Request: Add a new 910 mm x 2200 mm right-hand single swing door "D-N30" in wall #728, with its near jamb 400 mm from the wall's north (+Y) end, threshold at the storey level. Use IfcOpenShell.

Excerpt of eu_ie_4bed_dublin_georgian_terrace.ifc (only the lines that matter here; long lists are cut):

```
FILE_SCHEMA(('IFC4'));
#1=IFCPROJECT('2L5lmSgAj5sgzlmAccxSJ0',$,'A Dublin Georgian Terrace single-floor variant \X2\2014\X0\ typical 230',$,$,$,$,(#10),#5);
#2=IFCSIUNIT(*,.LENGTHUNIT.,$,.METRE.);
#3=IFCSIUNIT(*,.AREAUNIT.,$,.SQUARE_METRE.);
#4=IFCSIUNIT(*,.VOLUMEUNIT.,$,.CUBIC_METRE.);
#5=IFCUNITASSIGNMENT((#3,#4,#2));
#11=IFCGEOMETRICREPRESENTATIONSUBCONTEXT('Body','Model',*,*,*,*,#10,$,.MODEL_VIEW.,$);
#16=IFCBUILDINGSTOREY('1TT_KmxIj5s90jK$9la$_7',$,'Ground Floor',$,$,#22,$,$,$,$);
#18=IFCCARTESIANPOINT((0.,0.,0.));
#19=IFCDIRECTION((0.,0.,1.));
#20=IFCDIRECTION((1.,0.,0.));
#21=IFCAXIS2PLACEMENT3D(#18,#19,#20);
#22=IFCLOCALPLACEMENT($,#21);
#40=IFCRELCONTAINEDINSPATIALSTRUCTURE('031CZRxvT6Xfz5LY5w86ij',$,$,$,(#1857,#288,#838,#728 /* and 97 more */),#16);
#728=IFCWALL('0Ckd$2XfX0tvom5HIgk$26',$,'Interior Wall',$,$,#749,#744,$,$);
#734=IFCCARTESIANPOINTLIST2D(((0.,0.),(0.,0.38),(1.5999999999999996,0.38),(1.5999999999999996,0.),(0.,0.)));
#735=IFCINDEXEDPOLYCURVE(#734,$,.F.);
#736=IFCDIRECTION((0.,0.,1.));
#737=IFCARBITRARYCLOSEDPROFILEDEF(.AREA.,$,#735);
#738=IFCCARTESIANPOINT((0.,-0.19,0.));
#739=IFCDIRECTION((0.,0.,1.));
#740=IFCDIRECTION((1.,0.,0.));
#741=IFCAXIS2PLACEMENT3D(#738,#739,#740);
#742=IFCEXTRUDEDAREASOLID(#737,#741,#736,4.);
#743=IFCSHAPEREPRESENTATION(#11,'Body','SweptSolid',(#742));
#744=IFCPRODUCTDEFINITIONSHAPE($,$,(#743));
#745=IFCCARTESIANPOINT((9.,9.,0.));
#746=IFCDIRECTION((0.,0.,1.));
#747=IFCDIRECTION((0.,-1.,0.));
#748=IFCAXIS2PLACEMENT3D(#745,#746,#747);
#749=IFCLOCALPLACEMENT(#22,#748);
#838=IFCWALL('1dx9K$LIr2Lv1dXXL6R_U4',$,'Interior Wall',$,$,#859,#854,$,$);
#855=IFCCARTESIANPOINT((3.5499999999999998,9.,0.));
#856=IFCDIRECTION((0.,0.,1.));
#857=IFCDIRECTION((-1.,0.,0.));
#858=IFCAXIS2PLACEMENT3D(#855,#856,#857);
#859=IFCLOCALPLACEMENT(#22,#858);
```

```python
import numpy as np
import ifcopenshell
import ifcopenshell.api.feature
import ifcopenshell.api.geometry
import ifcopenshell.api.root
import ifcopenshell.api.spatial
import ifcopenshell.geom
import ifcopenshell.util.element
import ifcopenshell.util.placement
import ifcopenshell.util.representation
import ifcopenshell.util.shape
import ifcopenshell.util.unit

model = ifcopenshell.open("eu_ie_4bed_dublin_georgian_terrace.ifc")
unit_scale = ifcopenshell.util.unit.calculate_unit_scale(model)
settings = ifcopenshell.geom.settings()


def volume(element):
    """Net volume in cubic metres, openings subtracted."""
    shape = ifcopenshell.geom.create_shape(settings, element)
    return ifcopenshell.util.shape.get_volume(shape.geometry)


wall = model.by_guid("0Ckd$2XfX0tvom5HIgk$26")
storey = ifcopenshell.util.element.get_container(wall, ifc_class="IfcBuildingStorey")
context = ifcopenshell.util.representation.get_context(model, "Model", "Body", "MODEL_VIEW")
before = volume(wall)

width, height, from_end, sill = 0.91, 2.2, 0.4, 0.0  # metres

# The wall runs along its own X axis, and the end named is its -X end.
wall_shape = ifcopenshell.geom.create_shape(settings, wall)
x, y, z = ifcopenshell.util.shape.get_vertices(wall_shape.geometry).T
start = x.min() + from_end
face, thickness = float(y.min()), float(y.max() - y.min())
wall_matrix = ifcopenshell.util.placement.get_local_placement(wall.ObjectPlacement)
level = ifcopenshell.util.placement.get_local_placement(storey.ObjectPlacement)[2, 3]


def in_wall(x, y):
    """Placement at x, y metres in the wall's axes, at sill height."""
    matrix = wall_matrix.copy()
    matrix[:, 3] = wall_matrix @ np.array([x / unit_scale, y / unit_scale, 0.0, 1.0])
    matrix[2, 3] = level + sill / unit_scale
    return matrix


# Opening: a box that overshoots both wall faces by 50 mm.
opening = ifcopenshell.api.root.create_entity(model, ifc_class="IfcOpeningElement", predefined_type="OPENING")
box = ifcopenshell.api.geometry.add_wall_representation(
    model, context=context, length=width, height=height, thickness=thickness + 0.1
)
ifcopenshell.api.geometry.assign_representation(model, product=opening, representation=box)
ifcopenshell.api.geometry.edit_object_placement(model, product=opening, matrix=in_wall(start, face - 0.05), is_si=False)
ifcopenshell.api.feature.add_feature(model, feature=opening, element=wall)

door = ifcopenshell.api.root.create_entity(model, ifc_class="IfcDoor", name="D-N30", predefined_type="DOOR")
door.OverallWidth, door.OverallHeight = width / unit_scale, height / unit_scale
door.OperationType = "SINGLE_SWING_RIGHT"
body = ifcopenshell.api.geometry.add_door_representation(
    model,
    context=context,
    overall_width=door.OverallWidth,
    overall_height=door.OverallHeight,
    operation_type="SINGLE_SWING_RIGHT",
    lining_properties={"LiningDepth": thickness / unit_scale, "ThresholdDepth": thickness / unit_scale},
)
ifcopenshell.api.geometry.assign_representation(model, product=door, representation=body)
ifcopenshell.api.spatial.assign_container(model, products=[door], relating_structure=storey)
ifcopenshell.api.feature.add_filling(model, opening=opening, element=door)

# The lining spans the wall, so the door starts at the wall face.
ifcopenshell.api.geometry.edit_object_placement(model, product=door, matrix=in_wall(start, face), is_si=False)

after = volume(wall)

print(f"wall volume {before:.3f} -> {after:.3f} m3")

model.write("eu_ie_4bed_dublin_georgian_terrace_updated.ifc")
```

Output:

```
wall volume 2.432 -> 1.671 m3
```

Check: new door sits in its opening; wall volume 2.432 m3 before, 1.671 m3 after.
